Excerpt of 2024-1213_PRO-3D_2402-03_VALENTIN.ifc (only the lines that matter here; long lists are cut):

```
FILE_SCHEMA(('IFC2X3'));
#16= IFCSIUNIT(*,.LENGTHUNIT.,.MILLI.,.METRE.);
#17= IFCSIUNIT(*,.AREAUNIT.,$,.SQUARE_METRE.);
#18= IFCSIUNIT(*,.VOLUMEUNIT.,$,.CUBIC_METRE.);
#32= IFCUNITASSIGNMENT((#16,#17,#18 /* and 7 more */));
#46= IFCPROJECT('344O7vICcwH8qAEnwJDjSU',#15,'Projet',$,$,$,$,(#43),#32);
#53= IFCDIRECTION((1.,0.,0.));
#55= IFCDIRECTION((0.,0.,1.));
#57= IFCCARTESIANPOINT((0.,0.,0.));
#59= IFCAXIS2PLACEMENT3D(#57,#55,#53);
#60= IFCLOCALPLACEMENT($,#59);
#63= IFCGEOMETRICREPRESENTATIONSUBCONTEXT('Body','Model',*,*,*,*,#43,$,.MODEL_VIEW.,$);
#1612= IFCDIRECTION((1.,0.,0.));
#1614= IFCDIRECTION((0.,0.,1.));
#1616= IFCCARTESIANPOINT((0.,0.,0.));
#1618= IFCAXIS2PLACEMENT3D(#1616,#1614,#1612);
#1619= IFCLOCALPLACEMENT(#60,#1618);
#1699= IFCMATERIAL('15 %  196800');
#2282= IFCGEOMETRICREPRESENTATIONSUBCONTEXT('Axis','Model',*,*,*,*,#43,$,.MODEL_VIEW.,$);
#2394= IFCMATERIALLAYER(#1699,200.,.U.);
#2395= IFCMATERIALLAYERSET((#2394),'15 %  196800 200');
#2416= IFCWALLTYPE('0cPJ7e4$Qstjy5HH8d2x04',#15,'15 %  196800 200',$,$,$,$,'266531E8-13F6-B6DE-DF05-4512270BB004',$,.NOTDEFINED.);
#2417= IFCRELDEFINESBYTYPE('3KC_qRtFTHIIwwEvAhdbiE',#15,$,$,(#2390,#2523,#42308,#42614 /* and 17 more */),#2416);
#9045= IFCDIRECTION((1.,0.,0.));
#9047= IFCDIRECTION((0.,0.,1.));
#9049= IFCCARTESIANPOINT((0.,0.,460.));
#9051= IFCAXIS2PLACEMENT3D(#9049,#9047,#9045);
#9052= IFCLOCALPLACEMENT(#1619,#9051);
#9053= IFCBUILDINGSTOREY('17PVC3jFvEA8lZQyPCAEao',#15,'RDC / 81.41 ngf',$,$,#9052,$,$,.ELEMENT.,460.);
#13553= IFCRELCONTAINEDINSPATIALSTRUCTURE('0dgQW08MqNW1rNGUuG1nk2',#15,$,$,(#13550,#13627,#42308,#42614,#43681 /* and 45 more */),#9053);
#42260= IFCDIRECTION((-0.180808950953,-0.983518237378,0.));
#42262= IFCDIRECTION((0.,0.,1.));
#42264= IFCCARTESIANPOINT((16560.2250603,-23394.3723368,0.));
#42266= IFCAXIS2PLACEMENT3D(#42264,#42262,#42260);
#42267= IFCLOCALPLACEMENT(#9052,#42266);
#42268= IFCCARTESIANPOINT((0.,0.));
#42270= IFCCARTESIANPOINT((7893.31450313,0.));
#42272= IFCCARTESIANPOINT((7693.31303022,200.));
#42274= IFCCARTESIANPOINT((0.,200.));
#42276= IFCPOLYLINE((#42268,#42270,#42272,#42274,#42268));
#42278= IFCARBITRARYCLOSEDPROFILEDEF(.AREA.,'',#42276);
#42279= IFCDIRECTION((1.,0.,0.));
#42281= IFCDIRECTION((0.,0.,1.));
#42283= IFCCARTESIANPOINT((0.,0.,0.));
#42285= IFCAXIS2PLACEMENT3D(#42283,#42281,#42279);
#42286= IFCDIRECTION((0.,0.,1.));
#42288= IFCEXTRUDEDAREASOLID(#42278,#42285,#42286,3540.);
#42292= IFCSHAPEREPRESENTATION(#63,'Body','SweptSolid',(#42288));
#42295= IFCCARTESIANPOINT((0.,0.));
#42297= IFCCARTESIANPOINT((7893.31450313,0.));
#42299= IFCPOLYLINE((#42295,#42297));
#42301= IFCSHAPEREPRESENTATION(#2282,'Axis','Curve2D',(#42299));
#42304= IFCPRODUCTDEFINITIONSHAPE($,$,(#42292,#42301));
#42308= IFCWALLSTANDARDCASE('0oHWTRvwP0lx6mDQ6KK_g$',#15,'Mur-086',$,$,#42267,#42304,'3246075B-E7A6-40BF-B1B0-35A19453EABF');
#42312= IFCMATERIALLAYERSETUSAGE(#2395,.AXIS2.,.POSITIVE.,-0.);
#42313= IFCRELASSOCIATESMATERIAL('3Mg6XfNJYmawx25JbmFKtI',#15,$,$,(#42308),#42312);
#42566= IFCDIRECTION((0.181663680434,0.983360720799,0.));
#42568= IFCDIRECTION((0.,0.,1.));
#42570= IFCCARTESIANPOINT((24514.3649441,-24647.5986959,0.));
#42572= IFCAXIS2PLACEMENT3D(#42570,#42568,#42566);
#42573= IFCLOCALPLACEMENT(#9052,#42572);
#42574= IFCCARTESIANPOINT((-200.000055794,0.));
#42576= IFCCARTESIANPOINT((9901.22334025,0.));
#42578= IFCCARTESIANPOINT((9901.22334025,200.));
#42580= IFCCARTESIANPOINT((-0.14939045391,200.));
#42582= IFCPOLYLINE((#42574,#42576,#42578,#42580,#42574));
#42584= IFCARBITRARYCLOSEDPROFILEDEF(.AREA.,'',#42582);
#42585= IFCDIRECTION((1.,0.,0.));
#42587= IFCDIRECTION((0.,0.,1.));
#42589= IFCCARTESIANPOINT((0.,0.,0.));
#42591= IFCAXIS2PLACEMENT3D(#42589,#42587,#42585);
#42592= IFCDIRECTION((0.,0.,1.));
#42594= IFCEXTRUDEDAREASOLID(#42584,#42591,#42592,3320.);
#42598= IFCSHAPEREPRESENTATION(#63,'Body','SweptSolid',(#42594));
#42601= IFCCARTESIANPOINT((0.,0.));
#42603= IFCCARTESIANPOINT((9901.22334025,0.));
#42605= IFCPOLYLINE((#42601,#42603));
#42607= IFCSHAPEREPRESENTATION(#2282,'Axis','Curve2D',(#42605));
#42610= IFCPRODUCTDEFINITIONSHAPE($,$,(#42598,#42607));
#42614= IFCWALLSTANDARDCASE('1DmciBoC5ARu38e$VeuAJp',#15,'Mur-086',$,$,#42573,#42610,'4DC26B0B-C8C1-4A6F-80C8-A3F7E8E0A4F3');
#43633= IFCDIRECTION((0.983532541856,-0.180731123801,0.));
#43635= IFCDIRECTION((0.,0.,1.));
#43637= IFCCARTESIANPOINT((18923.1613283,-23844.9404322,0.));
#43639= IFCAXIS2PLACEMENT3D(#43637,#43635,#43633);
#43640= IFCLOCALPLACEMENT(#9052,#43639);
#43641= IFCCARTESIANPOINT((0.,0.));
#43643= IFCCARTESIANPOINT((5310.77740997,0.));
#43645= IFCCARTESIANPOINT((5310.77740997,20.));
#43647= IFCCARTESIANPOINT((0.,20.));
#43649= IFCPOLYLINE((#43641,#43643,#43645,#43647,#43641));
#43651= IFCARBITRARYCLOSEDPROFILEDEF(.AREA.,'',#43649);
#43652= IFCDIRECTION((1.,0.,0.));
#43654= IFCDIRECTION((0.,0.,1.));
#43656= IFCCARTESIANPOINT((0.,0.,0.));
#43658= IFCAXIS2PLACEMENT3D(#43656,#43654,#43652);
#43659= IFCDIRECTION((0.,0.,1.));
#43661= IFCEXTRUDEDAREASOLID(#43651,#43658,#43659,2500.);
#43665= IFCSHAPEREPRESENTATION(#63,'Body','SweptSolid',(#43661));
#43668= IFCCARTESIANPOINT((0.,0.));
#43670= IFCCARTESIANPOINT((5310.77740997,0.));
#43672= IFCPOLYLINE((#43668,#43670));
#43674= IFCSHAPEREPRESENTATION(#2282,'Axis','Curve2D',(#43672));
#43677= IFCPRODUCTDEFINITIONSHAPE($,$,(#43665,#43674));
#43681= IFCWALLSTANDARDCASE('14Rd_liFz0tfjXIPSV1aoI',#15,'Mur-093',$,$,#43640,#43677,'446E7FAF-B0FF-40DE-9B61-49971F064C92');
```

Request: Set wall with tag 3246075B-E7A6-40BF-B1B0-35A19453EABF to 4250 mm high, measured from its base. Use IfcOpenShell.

```python
import ifcopenshell
import ifcopenshell.geom
import ifcopenshell.util.representation
import ifcopenshell.util.shape

model = ifcopenshell.open("2024-1213_PRO-3D_2402-03_VALENTIN.ifc")
settings = ifcopenshell.geom.settings()


def volume(element):
    """Net volume in cubic metres, openings subtracted."""
    shape = ifcopenshell.geom.create_shape(settings, element)
    return ifcopenshell.util.shape.get_volume(shape.geometry)


wall = model.by_id(42308)
before = volume(wall)

body = ifcopenshell.util.representation.get_representation(wall, "Model", "Body")
solid = body.Items[0]
old_height = solid.Depth
solid.Depth = 4250.0
after = volume(wall)

print(f"height {old_height:g} -> {solid.Depth:g}, volume {before:.3f} -> {after:.3f} m3")

model.write("2024-1213_PRO-3D_2402-03_VALENTIN_v2.ifc")
```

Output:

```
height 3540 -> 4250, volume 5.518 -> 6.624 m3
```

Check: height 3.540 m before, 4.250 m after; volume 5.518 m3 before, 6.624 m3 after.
